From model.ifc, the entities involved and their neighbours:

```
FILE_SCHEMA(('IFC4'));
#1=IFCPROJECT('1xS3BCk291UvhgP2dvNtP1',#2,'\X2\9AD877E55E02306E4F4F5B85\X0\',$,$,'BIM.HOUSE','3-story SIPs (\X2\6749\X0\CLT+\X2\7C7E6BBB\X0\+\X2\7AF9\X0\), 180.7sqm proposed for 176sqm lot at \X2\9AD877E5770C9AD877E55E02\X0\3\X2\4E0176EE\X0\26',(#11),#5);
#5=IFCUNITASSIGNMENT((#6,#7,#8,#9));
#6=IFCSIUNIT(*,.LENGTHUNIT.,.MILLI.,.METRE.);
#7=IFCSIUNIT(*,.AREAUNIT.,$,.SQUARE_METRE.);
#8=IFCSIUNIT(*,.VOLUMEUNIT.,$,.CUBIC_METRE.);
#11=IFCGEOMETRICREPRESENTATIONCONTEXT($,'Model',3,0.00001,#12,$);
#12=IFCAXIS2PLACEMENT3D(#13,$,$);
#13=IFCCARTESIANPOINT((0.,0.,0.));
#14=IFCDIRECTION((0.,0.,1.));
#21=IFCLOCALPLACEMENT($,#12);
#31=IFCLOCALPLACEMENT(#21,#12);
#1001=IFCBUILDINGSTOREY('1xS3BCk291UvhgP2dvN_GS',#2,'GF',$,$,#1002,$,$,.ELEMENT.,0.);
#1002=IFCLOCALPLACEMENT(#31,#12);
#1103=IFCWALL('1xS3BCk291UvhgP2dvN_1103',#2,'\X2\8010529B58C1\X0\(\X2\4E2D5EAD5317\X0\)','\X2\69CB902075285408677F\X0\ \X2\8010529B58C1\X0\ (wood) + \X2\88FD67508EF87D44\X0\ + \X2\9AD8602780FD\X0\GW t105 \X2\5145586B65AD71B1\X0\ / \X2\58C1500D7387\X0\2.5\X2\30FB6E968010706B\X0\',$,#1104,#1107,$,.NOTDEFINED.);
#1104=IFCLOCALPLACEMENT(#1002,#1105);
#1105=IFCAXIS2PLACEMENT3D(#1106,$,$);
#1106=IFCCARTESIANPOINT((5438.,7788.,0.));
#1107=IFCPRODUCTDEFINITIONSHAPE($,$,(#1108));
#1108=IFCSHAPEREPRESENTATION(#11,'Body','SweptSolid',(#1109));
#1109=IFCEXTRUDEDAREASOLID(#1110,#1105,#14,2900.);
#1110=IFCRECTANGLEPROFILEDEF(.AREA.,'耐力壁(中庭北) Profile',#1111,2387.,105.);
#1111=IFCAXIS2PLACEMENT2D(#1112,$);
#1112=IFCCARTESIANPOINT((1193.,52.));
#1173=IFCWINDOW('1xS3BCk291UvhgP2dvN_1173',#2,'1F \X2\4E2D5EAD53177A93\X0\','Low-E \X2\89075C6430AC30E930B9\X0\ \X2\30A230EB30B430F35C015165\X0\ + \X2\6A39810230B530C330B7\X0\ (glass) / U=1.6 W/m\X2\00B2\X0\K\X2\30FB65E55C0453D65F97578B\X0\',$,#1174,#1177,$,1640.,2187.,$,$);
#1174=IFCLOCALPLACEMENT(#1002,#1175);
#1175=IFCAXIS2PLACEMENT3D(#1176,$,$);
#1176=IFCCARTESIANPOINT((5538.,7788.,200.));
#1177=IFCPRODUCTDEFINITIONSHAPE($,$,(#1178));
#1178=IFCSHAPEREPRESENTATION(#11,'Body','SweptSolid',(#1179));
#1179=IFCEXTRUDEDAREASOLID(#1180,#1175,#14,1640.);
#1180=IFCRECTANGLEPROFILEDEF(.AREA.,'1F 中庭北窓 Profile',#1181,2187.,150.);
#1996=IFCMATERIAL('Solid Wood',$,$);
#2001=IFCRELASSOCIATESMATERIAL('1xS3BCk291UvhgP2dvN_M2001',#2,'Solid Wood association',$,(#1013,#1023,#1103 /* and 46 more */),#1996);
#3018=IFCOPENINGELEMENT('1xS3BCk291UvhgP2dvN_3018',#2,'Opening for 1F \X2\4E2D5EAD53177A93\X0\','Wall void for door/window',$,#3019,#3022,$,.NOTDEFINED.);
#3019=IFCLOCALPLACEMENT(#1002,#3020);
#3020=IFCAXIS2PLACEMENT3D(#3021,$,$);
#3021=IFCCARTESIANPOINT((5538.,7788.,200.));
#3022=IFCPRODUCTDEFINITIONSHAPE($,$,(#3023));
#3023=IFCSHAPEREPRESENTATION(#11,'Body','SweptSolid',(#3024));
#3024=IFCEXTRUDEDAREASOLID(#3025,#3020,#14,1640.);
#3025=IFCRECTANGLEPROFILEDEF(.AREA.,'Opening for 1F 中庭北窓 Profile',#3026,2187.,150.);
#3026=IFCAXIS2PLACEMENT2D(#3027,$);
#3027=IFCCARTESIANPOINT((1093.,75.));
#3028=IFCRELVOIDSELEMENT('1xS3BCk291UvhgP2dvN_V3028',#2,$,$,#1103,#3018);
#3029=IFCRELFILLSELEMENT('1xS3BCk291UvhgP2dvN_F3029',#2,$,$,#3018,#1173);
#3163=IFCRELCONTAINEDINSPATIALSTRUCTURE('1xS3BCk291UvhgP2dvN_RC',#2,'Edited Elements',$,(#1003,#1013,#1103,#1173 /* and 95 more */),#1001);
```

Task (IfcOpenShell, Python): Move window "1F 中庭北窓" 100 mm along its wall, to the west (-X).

```python
import ifcopenshell
import ifcopenshell.api.geometry
import ifcopenshell.util.placement
import ifcopenshell.util.unit

model = ifcopenshell.open("model.ifc")
unit_scale = ifcopenshell.util.unit.calculate_unit_scale(model)

window = model.by_guid("1xS3BCk291UvhgP2dvN_1173")
opening = window.FillsVoids[0].RelatingOpeningElement
wall = opening.VoidsElements[0].RelatingBuildingElement

wall_matrix = ifcopenshell.util.placement.get_local_placement(wall.ObjectPlacement)
shift = wall_matrix[:3, 0] * -0.1 / unit_scale
before = ifcopenshell.util.placement.get_local_placement(window.ObjectPlacement)[:3, 3].copy()

# The window is not placed relative to its opening, so move both.
for product in (opening, window):
    matrix = ifcopenshell.util.placement.get_local_placement(product.ObjectPlacement)
    matrix[:3, 3] += shift
    ifcopenshell.api.geometry.edit_object_placement(model, product=product, matrix=matrix, is_si=False)

after = ifcopenshell.util.placement.get_local_placement(window.ObjectPlacement)[:3, 3]
print("window moved by", (after - before).round(3) + 0.0)

model.write("model_v2.ifc")
```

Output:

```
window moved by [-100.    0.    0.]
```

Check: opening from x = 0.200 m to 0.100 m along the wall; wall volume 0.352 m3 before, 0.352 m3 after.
